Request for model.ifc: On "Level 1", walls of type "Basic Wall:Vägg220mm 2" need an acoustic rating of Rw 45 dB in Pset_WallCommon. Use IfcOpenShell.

First a look at what the model holds.

```python
import ifcopenshell
import ifcopenshell.util.element

model = ifcopenshell.open("model.ifc")
print(model.schema)
storey = next(s for s in model.by_type("IfcBuildingStorey") if s.Name == "Level 1")
walls = [e for e in ifcopenshell.util.element.get_decomposition(storey) if e.is_a("IfcWall")]
seen = {}
for e in walls:
    element_type = ifcopenshell.util.element.get_type(e)
    key = (element_type.Name if element_type != e and element_type else None, ifcopenshell.util.element.get_pset(e, "Pset_WallCommon", "AcousticRating"))
    seen[key] = seen.get(key, 0) + 1
for (name, value), count in sorted(seen.items(), key=str):
    print(count, "x", name, "|", value)
```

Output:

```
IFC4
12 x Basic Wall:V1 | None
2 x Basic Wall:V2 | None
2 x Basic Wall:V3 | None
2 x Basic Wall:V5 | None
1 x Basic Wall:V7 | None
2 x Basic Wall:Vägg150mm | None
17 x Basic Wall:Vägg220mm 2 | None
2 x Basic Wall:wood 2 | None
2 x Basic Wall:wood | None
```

```python
import ifcopenshell
import ifcopenshell.api.pset
import ifcopenshell.util.element

model = ifcopenshell.open("model.ifc")

storey = next(s for s in model.by_type("IfcBuildingStorey") if s.Name == "Level 1")
walls = [e for e in ifcopenshell.util.element.get_decomposition(storey) if e.is_a("IfcWall")]

count = 0
for e in walls:
    element_type = ifcopenshell.util.element.get_type(e)
    if element_type in (None, e) or element_type.Name != "Basic Wall:Vägg220mm 2":
        continue
    # add_pset returns the element's existing set when there is one.
    pset = ifcopenshell.api.pset.add_pset(model, product=e, name="Pset_WallCommon")
    ifcopenshell.api.pset.edit_pset(model, pset=pset, properties={"AcousticRating": "Rw 45 dB"})
    count += 1

print(count, "walls updated")

model.write("model_rev.ifc")
```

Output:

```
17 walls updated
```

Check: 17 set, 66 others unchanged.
